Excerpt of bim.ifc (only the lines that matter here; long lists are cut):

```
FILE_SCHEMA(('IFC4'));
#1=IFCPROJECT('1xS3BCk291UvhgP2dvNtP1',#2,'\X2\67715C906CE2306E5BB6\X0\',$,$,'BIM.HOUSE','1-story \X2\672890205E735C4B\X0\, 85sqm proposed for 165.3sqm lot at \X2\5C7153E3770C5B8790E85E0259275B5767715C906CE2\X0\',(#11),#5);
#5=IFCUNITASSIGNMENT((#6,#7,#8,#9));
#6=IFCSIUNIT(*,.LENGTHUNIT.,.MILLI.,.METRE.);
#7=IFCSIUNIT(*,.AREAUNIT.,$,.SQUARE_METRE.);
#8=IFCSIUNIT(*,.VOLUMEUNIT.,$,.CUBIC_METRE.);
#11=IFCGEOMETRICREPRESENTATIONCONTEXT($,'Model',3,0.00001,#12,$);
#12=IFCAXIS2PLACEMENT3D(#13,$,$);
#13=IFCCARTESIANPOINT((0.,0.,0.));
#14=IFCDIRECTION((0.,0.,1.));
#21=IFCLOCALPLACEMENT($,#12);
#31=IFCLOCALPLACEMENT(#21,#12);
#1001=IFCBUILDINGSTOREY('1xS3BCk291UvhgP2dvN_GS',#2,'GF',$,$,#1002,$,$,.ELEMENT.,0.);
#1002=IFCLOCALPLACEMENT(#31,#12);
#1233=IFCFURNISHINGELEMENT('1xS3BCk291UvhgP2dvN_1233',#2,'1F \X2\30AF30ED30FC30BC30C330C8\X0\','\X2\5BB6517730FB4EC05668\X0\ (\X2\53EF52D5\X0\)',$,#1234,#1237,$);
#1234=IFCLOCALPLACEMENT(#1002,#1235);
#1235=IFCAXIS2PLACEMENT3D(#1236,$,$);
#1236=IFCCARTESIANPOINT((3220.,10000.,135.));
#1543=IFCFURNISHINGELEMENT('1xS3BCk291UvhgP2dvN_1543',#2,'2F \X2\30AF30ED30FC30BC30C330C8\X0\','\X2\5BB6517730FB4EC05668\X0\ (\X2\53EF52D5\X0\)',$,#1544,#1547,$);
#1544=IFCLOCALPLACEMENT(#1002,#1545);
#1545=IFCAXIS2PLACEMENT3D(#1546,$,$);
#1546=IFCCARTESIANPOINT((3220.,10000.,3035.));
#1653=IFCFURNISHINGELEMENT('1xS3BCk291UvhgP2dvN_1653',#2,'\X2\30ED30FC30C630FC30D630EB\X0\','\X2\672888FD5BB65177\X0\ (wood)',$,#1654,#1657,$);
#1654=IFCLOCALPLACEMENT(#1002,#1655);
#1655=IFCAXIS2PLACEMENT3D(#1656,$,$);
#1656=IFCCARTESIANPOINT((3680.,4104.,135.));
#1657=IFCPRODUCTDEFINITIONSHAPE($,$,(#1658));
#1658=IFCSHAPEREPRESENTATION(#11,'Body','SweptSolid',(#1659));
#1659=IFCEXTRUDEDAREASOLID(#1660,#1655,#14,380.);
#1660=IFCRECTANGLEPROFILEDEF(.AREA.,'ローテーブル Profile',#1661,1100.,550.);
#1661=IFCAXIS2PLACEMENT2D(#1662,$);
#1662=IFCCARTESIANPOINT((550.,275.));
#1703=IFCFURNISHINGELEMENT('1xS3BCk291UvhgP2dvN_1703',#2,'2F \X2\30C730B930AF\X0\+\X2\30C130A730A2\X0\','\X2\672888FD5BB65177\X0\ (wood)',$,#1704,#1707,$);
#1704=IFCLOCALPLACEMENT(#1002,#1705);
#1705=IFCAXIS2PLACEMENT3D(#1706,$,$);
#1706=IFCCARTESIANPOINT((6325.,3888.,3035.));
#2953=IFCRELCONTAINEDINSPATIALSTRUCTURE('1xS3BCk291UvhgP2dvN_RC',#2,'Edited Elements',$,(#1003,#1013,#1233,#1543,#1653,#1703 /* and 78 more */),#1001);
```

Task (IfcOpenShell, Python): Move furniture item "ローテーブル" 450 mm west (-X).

```python
import ifcopenshell
import ifcopenshell.api.geometry
import ifcopenshell.util.placement
import ifcopenshell.util.unit

model = ifcopenshell.open("bim.ifc")
unit_scale = ifcopenshell.util.unit.calculate_unit_scale(model)

item = model.by_id(1653)
matrix = ifcopenshell.util.placement.get_local_placement(item.ObjectPlacement)
matrix[0, 3] -= 0.45 / unit_scale
ifcopenshell.api.geometry.edit_object_placement(model, product=item, matrix=matrix, is_si=False)

print(ifcopenshell.util.placement.get_local_placement(item.ObjectPlacement).round(3) + 0.0)

model.write("bim_rev.ifc")
```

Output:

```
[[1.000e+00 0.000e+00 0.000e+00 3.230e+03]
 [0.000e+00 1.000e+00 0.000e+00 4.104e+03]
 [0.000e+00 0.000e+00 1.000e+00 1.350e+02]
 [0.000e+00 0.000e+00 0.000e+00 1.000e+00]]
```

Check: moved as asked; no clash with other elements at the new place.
